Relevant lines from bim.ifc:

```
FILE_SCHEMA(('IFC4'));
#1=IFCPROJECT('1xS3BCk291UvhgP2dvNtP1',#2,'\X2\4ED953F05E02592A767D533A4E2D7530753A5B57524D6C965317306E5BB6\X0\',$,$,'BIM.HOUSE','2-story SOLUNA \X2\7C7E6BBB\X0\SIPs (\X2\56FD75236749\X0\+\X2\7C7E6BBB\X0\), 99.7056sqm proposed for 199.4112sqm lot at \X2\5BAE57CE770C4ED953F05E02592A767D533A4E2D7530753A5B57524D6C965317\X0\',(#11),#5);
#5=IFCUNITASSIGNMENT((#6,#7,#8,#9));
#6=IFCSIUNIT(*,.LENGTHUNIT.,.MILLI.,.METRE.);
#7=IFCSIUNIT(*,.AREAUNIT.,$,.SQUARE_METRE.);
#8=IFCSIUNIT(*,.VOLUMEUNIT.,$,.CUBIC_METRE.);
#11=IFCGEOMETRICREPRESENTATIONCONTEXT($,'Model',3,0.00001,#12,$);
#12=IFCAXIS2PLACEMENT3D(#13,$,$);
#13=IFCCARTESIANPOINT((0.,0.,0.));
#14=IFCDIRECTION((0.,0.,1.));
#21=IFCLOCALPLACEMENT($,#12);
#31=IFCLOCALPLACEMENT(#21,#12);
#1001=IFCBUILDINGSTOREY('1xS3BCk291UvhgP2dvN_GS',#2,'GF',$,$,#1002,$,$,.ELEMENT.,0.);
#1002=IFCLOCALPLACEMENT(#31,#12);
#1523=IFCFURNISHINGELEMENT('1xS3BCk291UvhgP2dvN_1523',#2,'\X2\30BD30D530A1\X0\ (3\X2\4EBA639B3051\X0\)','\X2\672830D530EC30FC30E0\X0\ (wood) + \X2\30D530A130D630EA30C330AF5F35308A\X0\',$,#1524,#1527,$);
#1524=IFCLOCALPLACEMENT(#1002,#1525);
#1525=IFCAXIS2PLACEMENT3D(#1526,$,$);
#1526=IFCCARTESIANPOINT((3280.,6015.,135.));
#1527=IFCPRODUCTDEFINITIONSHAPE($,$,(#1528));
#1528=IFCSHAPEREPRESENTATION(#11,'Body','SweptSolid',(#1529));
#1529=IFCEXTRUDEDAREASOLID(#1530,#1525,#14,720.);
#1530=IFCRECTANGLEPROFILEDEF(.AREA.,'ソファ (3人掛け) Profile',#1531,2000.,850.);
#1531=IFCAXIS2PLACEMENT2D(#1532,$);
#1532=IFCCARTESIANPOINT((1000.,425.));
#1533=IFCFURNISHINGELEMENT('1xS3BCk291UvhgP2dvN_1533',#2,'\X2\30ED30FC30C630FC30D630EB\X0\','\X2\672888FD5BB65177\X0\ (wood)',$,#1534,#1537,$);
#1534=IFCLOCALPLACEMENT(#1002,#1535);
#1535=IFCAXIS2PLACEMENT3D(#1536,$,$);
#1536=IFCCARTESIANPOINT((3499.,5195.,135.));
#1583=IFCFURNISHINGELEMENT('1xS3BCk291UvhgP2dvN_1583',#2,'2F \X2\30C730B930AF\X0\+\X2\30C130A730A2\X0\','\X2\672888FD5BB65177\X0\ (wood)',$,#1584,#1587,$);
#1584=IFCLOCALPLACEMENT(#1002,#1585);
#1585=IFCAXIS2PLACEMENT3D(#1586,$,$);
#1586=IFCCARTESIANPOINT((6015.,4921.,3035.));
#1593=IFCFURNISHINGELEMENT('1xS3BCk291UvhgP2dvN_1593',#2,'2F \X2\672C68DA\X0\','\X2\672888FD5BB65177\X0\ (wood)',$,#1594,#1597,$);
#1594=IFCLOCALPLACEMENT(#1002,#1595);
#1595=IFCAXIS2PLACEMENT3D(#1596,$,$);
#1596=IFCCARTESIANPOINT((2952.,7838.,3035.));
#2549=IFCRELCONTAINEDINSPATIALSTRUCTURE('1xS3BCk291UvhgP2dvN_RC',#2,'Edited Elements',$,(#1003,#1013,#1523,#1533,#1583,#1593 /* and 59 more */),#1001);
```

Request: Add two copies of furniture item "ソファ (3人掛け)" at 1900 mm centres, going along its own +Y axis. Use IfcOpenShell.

```python
import ifcopenshell
import ifcopenshell.api.geometry
import ifcopenshell.api.root
import ifcopenshell.util.element
import ifcopenshell.util.placement
import ifcopenshell.util.unit

model = ifcopenshell.open("bim.ifc")
unit_scale = ifcopenshell.util.unit.calculate_unit_scale(model)


def reuse_history(source, copy):
    """copy_class also copies each property set's owner history, people and application; keep the originals."""
    for rel in copy.IsDefinedBy:
        if rel.is_a("IfcRelDefinesByProperties") and (history := rel.RelatingPropertyDefinition.OwnerHistory):
            rel.RelatingPropertyDefinition.OwnerHistory = source.OwnerHistory
            ifcopenshell.util.element.remove_deep2(model, history)


source = model.by_guid("1xS3BCk291UvhgP2dvN_1523")
base = ifcopenshell.util.placement.get_local_placement(source.ObjectPlacement)
step = base[:3, 1] * 1.9 / unit_scale

for i in range(1, 3):
    copy = ifcopenshell.api.root.copy_class(model, product=source)
    copy.Representation = ifcopenshell.util.element.copy_deep(
        model, source.Representation, exclude=["IfcGeometricRepresentationContext", "IfcRepresentationMap"]
    )
    reuse_history(source, copy)
    matrix = base.copy()
    matrix[:3, 3] += i * step
    print("added at", matrix[:3, 3].round(3) + 0.0)
    ifcopenshell.api.geometry.edit_object_placement(model, product=copy, matrix=matrix, is_si=False)

model.write("bim_updated.ifc")
```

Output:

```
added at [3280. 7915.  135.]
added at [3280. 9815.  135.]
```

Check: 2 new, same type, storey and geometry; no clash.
